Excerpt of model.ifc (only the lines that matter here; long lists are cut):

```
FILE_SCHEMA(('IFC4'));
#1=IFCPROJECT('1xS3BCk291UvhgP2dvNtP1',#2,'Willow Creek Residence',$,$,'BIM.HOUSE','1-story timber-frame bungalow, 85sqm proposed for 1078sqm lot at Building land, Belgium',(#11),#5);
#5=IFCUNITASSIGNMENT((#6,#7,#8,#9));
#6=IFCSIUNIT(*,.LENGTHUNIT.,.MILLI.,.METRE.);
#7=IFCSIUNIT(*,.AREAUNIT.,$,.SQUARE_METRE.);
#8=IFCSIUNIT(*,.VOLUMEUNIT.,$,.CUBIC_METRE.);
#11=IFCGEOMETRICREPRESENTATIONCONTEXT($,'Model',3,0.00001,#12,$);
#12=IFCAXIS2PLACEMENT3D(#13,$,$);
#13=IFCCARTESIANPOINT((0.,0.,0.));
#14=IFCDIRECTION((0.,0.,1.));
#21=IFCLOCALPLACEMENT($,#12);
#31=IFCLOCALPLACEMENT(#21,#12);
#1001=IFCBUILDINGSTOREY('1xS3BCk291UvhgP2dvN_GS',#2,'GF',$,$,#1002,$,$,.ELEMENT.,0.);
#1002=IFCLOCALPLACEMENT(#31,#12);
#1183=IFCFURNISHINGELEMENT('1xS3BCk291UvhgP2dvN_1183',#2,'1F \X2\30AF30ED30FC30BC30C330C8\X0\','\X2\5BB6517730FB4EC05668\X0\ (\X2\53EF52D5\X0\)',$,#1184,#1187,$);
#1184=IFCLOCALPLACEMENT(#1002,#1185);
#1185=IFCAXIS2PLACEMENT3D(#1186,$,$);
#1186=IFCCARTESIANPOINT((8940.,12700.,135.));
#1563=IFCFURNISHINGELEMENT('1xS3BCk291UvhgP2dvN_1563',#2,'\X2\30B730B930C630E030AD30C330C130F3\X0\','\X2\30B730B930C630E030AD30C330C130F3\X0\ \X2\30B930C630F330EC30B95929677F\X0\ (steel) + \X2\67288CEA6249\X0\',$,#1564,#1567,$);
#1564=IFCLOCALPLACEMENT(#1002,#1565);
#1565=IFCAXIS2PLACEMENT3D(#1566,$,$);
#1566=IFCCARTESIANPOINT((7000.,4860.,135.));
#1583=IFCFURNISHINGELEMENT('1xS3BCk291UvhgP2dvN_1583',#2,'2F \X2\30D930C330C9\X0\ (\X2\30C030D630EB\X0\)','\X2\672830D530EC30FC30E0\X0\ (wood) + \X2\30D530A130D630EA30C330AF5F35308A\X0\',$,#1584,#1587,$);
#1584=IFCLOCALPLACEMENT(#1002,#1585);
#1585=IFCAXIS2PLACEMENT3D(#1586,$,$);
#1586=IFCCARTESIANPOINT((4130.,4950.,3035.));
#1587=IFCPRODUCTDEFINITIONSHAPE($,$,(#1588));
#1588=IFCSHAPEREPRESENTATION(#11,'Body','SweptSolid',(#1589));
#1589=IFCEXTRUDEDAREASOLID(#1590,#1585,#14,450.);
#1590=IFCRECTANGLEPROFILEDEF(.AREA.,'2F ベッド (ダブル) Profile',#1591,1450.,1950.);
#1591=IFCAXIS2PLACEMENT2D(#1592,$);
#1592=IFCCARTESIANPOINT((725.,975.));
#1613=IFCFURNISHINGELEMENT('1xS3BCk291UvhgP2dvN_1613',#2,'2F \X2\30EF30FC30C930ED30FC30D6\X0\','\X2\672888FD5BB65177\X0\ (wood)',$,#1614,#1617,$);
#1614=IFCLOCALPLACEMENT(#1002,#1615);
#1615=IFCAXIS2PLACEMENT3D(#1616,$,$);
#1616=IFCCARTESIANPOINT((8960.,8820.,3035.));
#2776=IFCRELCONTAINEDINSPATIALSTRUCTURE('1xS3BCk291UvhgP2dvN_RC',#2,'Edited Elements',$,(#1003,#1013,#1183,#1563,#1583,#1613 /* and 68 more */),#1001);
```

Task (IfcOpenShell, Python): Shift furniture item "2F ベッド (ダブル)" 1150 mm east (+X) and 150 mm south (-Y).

```python
import ifcopenshell
import ifcopenshell.api.geometry
import ifcopenshell.util.placement
import ifcopenshell.util.unit

model = ifcopenshell.open("model.ifc")
unit_scale = ifcopenshell.util.unit.calculate_unit_scale(model)

item = model.by_guid("1xS3BCk291UvhgP2dvN_1583")
matrix = ifcopenshell.util.placement.get_local_placement(item.ObjectPlacement)
matrix[0, 3] += 1.15 / unit_scale
matrix[1, 3] -= 0.15 / unit_scale
ifcopenshell.api.geometry.edit_object_placement(model, product=item, matrix=matrix, is_si=False)

print(ifcopenshell.util.placement.get_local_placement(item.ObjectPlacement).round(3) + 0.0)

model.write("model_v2.ifc")
```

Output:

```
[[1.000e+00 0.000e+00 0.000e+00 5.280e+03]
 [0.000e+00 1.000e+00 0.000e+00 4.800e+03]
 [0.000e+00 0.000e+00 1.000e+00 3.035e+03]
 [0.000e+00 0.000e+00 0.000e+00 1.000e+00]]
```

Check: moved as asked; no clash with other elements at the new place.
